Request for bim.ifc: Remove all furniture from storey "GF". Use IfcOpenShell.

First a look at what the model holds.

```python
import ifcopenshell
import ifcopenshell.util.element

model = ifcopenshell.open("bim.ifc")
print(model.schema)
storey = next(s for s in model.by_type("IfcBuildingStorey") if s.Name == "GF")
furniture = [e for e in ifcopenshell.util.element.get_decomposition(storey) if e.is_a("IfcFurnishingElement")]
seen = {}
for e in furniture:
    element_type = ifcopenshell.util.element.get_type(e)
    name = element_type.Name if element_type not in (None, e) else None
    seen[name] = seen.get(name, 0) + 1
for name, count in sorted(seen.items(), key=str):
    print(count, "x", name)
```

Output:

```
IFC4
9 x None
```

```python
import ifcopenshell
import ifcopenshell.api.root
import ifcopenshell.util.element

model = ifcopenshell.open("bim.ifc")

storey = next(s for s in model.by_type("IfcBuildingStorey") if s.Name == "GF")
furniture = [e for e in ifcopenshell.util.element.get_decomposition(storey) if e.is_a("IfcFurnishingElement")]

for e in furniture:
    ifcopenshell.api.root.remove_product(model, product=e)
print(len(furniture), "removed")

model.write("bim_v2.ifc")
```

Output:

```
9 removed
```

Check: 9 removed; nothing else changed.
